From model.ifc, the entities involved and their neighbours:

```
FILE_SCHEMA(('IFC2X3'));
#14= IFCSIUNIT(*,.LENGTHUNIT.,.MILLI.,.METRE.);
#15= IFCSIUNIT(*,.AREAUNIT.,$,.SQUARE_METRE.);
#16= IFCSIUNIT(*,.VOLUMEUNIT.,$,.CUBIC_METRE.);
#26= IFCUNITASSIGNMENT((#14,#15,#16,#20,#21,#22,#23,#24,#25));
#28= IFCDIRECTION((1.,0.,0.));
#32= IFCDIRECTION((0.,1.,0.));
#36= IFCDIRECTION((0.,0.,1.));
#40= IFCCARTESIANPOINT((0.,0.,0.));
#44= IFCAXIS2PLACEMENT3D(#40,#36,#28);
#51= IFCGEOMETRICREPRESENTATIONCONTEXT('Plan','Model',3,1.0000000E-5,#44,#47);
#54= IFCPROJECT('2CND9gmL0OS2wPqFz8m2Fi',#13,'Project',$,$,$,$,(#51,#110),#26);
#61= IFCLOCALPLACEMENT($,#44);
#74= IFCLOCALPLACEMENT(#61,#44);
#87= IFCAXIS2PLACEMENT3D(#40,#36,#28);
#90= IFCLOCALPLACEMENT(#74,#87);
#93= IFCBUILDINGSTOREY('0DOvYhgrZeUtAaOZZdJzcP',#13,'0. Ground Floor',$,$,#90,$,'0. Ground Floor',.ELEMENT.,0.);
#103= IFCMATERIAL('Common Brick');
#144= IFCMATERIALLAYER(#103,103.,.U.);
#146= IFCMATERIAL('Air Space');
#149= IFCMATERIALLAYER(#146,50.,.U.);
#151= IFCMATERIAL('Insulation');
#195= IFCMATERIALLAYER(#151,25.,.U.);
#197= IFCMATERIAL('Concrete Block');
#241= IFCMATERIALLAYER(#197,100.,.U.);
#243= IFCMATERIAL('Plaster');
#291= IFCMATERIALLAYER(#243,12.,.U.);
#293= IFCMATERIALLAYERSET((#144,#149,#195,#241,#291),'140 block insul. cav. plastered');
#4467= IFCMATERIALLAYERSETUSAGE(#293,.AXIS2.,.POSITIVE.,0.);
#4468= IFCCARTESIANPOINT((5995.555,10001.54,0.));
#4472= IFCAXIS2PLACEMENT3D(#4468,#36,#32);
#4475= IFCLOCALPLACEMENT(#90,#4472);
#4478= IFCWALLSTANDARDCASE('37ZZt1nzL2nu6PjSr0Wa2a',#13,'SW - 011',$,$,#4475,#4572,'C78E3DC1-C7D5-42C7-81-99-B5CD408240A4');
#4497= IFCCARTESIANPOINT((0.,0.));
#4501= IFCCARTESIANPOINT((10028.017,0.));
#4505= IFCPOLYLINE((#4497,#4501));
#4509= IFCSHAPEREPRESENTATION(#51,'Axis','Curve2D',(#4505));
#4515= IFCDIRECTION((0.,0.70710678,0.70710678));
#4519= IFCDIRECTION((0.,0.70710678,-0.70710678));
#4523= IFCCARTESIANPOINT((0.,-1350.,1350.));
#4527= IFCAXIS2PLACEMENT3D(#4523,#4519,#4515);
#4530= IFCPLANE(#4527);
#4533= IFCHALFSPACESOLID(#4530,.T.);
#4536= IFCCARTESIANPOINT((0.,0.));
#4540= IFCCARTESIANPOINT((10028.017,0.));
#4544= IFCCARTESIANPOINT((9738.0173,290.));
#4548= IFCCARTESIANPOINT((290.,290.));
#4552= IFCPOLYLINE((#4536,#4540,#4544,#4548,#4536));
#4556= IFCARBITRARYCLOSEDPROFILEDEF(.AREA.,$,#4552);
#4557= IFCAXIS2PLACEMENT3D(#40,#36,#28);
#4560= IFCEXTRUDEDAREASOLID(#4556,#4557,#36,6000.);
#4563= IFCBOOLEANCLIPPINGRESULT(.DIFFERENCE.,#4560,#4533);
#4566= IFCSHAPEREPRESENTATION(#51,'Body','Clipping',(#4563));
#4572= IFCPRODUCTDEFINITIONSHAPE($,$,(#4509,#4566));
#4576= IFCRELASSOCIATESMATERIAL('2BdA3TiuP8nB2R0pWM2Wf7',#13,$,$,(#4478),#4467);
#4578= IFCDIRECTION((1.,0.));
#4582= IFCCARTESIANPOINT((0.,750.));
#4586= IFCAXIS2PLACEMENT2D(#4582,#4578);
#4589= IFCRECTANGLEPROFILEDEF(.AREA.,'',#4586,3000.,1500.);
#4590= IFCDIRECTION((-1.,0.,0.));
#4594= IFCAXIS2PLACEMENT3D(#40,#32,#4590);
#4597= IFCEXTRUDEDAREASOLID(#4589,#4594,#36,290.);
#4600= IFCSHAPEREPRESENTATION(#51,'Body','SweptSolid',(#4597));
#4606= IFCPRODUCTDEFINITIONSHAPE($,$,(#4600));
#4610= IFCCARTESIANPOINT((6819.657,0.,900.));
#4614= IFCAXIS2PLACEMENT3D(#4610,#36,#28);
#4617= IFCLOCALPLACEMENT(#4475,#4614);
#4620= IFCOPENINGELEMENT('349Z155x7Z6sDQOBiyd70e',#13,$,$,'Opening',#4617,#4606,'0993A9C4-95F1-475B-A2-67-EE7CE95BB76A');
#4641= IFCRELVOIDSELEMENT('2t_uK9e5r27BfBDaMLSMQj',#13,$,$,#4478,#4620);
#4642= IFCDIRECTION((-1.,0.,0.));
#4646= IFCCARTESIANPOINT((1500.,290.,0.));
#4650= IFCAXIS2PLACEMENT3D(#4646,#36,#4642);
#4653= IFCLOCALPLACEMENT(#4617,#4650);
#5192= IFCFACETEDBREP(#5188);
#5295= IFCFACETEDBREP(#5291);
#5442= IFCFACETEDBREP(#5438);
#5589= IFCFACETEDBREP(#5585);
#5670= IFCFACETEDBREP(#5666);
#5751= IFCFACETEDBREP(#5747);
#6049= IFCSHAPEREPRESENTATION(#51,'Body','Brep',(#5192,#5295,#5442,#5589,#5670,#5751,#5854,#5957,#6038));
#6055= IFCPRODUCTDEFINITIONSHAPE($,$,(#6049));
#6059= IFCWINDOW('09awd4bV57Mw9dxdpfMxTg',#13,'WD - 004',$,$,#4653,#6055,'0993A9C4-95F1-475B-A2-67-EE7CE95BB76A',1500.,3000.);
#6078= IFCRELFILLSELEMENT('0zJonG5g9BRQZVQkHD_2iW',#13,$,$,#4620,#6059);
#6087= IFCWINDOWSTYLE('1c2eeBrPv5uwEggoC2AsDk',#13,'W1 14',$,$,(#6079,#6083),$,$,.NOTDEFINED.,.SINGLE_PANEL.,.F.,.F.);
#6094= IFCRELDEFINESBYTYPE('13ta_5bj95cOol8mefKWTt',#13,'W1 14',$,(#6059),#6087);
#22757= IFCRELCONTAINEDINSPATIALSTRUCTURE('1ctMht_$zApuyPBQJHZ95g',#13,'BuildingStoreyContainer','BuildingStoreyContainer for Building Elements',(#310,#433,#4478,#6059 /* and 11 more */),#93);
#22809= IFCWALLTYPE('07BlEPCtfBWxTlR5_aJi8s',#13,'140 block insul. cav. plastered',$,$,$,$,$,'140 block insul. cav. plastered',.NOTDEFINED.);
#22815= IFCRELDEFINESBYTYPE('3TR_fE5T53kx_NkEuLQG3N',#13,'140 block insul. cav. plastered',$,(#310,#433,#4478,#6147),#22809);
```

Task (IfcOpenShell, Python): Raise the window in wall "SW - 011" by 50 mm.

```python
import numpy as np
import ifcopenshell
import ifcopenshell.api.geometry
import ifcopenshell.util.placement
import ifcopenshell.util.unit

model = ifcopenshell.open("model.ifc")
unit_scale = ifcopenshell.util.unit.calculate_unit_scale(model)

window = model.by_id(6059)
opening = window.FillsVoids[0].RelatingOpeningElement
dz = 50.0

shift = np.array([0.0, 0.0, dz])
# The window is placed relative to its opening, so it follows when the opening moves.
matrix = ifcopenshell.util.placement.get_local_placement(opening.ObjectPlacement)
matrix[:3, 3] += shift
ifcopenshell.api.geometry.edit_object_placement(
    model, product=opening, matrix=matrix, is_si=False, should_transform_children=True
)

print(f"moved by {dz * unit_scale:+.3f} m")

model.write("model_v2.ifc")
```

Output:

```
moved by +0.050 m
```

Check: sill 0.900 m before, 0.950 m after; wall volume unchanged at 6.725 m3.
